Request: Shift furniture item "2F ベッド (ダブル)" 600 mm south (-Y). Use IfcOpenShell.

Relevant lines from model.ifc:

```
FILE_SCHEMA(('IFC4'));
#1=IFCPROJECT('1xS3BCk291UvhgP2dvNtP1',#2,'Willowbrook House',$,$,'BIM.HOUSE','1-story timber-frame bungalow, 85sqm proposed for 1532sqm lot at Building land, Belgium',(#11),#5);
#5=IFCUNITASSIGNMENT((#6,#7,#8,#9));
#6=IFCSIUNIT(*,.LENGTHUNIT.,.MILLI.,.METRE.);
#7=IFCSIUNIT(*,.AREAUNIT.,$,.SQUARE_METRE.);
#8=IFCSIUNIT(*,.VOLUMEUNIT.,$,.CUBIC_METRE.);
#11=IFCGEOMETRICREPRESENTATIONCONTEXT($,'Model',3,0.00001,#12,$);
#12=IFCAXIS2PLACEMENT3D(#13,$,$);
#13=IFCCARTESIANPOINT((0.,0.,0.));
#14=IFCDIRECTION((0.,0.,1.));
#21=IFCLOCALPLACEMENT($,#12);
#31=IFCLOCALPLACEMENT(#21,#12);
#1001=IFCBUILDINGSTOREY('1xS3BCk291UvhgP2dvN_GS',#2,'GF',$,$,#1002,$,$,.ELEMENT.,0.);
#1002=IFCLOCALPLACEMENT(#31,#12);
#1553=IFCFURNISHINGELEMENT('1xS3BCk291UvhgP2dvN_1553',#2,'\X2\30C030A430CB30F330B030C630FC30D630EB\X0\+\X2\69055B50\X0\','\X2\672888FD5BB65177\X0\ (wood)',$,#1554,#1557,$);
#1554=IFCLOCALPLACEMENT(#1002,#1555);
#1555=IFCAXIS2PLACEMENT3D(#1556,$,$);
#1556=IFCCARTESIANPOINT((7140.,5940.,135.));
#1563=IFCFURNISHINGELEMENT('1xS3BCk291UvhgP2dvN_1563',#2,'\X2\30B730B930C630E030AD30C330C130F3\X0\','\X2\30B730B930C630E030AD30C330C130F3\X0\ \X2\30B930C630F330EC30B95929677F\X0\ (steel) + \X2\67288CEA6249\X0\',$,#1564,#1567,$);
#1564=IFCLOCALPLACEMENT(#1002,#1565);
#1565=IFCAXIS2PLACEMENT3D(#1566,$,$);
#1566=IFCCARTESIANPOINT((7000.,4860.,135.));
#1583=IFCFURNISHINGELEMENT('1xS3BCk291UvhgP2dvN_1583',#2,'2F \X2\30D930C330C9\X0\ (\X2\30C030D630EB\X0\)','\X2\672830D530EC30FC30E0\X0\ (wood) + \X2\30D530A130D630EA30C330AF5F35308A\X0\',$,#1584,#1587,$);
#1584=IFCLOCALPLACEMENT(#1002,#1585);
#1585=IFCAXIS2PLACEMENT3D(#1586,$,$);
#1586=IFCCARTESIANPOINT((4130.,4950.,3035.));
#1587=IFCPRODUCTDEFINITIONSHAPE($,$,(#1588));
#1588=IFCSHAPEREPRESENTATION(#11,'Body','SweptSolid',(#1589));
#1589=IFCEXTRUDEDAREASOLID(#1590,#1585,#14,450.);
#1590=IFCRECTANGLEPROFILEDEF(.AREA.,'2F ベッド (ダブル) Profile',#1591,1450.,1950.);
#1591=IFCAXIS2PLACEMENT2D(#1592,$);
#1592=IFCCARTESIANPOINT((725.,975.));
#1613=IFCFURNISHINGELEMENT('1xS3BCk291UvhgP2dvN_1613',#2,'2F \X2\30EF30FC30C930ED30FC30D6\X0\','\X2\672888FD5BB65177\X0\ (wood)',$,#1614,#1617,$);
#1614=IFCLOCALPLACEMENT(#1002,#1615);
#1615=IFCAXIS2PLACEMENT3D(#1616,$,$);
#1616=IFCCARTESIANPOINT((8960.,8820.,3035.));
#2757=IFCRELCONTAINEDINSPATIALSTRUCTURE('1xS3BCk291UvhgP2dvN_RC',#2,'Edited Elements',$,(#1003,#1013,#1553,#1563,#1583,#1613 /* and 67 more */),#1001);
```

```python
import ifcopenshell
import ifcopenshell.api.geometry
import ifcopenshell.util.placement
import ifcopenshell.util.unit

model = ifcopenshell.open("model.ifc")
unit_scale = ifcopenshell.util.unit.calculate_unit_scale(model)

item = model.by_guid("1xS3BCk291UvhgP2dvN_1583")
matrix = ifcopenshell.util.placement.get_local_placement(item.ObjectPlacement)
matrix[1, 3] -= 0.6 / unit_scale
ifcopenshell.api.geometry.edit_object_placement(model, product=item, matrix=matrix, is_si=False)

print(ifcopenshell.util.placement.get_local_placement(item.ObjectPlacement).round(3) + 0.0)

model.write("model_edited.ifc")
```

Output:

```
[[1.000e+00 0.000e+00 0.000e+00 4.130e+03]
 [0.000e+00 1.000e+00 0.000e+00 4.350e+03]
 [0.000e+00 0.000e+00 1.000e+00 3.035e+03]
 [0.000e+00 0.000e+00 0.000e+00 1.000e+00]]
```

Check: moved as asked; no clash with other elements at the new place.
